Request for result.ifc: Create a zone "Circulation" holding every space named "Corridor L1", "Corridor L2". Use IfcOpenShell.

First a look at what the model holds.

```python
import ifcopenshell

model = ifcopenshell.open("result.ifc")
print(model.schema)
seen = {}
for space in model.by_type("IfcSpace"):
    seen[space.Name] = seen.get(space.Name, 0) + 1
for name, count in sorted(seen.items(), key=str):
    print(count, "x", name)
print("zones:", [z.Name for z in model.by_type("IfcZone")][:20])
```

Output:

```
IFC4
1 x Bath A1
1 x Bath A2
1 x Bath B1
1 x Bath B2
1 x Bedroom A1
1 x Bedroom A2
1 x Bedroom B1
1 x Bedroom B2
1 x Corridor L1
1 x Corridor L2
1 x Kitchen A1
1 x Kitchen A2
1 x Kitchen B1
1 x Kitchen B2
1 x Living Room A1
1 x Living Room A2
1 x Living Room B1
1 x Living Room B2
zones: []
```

```python
import ifcopenshell
import ifcopenshell.api.group
import ifcopenshell.api.root

model = ifcopenshell.open("result.ifc")

names = {"Corridor L1", "Corridor L2"}
spaces = [s for s in model.by_type("IfcSpace") if s.Name in names]

zone = ifcopenshell.api.root.create_entity(model, ifc_class="IfcZone", name="Circulation")
ifcopenshell.api.group.assign_group(model, products=spaces, group=zone)
print(len(spaces), "spaces in", zone.Name)

model.write("result_updated.ifc")
```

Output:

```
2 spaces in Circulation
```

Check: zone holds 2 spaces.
